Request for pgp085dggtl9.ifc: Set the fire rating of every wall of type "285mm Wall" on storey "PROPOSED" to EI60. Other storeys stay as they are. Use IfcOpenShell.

First a look at what the model holds.

```python
import ifcopenshell
import ifcopenshell.util.element

model = ifcopenshell.open("pgp085dggtl9.ifc")
print(model.schema)
storey = next(s for s in model.by_type("IfcBuildingStorey") if s.Name == "PROPOSED")
walls = [e for e in ifcopenshell.util.element.get_decomposition(storey) if e.is_a("IfcWall")]
seen = {}
for e in walls:
    element_type = ifcopenshell.util.element.get_type(e)
    key = (element_type.Name if element_type != e and element_type else None, ifcopenshell.util.element.get_pset(e, "Pset_WallCommon", "FireRating"))
    seen[key] = seen.get(key, 0) + 1
for (name, value), count in sorted(seen.items(), key=str):
    print(count, "x", name, "|", value)
```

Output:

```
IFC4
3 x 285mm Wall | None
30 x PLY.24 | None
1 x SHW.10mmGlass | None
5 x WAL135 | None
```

```python
import ifcopenshell
import ifcopenshell.api.pset
import ifcopenshell.util.element

model = ifcopenshell.open("pgp085dggtl9.ifc")

storey = next(s for s in model.by_type("IfcBuildingStorey") if s.Name == "PROPOSED")
walls = [e for e in ifcopenshell.util.element.get_decomposition(storey) if e.is_a("IfcWall")]

count = 0
for e in walls:
    element_type = ifcopenshell.util.element.get_type(e)
    if element_type in (None, e) or element_type.Name != "285mm Wall":
        continue
    # add_pset returns the element's existing set when there is one.
    pset = ifcopenshell.api.pset.add_pset(model, product=e, name="Pset_WallCommon")
    ifcopenshell.api.pset.edit_pset(model, pset=pset, properties={"FireRating": "EI60"})
    count += 1

print(count, "walls updated")

model.write("pgp085dggtl9_v2.ifc")
```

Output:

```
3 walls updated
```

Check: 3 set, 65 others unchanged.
